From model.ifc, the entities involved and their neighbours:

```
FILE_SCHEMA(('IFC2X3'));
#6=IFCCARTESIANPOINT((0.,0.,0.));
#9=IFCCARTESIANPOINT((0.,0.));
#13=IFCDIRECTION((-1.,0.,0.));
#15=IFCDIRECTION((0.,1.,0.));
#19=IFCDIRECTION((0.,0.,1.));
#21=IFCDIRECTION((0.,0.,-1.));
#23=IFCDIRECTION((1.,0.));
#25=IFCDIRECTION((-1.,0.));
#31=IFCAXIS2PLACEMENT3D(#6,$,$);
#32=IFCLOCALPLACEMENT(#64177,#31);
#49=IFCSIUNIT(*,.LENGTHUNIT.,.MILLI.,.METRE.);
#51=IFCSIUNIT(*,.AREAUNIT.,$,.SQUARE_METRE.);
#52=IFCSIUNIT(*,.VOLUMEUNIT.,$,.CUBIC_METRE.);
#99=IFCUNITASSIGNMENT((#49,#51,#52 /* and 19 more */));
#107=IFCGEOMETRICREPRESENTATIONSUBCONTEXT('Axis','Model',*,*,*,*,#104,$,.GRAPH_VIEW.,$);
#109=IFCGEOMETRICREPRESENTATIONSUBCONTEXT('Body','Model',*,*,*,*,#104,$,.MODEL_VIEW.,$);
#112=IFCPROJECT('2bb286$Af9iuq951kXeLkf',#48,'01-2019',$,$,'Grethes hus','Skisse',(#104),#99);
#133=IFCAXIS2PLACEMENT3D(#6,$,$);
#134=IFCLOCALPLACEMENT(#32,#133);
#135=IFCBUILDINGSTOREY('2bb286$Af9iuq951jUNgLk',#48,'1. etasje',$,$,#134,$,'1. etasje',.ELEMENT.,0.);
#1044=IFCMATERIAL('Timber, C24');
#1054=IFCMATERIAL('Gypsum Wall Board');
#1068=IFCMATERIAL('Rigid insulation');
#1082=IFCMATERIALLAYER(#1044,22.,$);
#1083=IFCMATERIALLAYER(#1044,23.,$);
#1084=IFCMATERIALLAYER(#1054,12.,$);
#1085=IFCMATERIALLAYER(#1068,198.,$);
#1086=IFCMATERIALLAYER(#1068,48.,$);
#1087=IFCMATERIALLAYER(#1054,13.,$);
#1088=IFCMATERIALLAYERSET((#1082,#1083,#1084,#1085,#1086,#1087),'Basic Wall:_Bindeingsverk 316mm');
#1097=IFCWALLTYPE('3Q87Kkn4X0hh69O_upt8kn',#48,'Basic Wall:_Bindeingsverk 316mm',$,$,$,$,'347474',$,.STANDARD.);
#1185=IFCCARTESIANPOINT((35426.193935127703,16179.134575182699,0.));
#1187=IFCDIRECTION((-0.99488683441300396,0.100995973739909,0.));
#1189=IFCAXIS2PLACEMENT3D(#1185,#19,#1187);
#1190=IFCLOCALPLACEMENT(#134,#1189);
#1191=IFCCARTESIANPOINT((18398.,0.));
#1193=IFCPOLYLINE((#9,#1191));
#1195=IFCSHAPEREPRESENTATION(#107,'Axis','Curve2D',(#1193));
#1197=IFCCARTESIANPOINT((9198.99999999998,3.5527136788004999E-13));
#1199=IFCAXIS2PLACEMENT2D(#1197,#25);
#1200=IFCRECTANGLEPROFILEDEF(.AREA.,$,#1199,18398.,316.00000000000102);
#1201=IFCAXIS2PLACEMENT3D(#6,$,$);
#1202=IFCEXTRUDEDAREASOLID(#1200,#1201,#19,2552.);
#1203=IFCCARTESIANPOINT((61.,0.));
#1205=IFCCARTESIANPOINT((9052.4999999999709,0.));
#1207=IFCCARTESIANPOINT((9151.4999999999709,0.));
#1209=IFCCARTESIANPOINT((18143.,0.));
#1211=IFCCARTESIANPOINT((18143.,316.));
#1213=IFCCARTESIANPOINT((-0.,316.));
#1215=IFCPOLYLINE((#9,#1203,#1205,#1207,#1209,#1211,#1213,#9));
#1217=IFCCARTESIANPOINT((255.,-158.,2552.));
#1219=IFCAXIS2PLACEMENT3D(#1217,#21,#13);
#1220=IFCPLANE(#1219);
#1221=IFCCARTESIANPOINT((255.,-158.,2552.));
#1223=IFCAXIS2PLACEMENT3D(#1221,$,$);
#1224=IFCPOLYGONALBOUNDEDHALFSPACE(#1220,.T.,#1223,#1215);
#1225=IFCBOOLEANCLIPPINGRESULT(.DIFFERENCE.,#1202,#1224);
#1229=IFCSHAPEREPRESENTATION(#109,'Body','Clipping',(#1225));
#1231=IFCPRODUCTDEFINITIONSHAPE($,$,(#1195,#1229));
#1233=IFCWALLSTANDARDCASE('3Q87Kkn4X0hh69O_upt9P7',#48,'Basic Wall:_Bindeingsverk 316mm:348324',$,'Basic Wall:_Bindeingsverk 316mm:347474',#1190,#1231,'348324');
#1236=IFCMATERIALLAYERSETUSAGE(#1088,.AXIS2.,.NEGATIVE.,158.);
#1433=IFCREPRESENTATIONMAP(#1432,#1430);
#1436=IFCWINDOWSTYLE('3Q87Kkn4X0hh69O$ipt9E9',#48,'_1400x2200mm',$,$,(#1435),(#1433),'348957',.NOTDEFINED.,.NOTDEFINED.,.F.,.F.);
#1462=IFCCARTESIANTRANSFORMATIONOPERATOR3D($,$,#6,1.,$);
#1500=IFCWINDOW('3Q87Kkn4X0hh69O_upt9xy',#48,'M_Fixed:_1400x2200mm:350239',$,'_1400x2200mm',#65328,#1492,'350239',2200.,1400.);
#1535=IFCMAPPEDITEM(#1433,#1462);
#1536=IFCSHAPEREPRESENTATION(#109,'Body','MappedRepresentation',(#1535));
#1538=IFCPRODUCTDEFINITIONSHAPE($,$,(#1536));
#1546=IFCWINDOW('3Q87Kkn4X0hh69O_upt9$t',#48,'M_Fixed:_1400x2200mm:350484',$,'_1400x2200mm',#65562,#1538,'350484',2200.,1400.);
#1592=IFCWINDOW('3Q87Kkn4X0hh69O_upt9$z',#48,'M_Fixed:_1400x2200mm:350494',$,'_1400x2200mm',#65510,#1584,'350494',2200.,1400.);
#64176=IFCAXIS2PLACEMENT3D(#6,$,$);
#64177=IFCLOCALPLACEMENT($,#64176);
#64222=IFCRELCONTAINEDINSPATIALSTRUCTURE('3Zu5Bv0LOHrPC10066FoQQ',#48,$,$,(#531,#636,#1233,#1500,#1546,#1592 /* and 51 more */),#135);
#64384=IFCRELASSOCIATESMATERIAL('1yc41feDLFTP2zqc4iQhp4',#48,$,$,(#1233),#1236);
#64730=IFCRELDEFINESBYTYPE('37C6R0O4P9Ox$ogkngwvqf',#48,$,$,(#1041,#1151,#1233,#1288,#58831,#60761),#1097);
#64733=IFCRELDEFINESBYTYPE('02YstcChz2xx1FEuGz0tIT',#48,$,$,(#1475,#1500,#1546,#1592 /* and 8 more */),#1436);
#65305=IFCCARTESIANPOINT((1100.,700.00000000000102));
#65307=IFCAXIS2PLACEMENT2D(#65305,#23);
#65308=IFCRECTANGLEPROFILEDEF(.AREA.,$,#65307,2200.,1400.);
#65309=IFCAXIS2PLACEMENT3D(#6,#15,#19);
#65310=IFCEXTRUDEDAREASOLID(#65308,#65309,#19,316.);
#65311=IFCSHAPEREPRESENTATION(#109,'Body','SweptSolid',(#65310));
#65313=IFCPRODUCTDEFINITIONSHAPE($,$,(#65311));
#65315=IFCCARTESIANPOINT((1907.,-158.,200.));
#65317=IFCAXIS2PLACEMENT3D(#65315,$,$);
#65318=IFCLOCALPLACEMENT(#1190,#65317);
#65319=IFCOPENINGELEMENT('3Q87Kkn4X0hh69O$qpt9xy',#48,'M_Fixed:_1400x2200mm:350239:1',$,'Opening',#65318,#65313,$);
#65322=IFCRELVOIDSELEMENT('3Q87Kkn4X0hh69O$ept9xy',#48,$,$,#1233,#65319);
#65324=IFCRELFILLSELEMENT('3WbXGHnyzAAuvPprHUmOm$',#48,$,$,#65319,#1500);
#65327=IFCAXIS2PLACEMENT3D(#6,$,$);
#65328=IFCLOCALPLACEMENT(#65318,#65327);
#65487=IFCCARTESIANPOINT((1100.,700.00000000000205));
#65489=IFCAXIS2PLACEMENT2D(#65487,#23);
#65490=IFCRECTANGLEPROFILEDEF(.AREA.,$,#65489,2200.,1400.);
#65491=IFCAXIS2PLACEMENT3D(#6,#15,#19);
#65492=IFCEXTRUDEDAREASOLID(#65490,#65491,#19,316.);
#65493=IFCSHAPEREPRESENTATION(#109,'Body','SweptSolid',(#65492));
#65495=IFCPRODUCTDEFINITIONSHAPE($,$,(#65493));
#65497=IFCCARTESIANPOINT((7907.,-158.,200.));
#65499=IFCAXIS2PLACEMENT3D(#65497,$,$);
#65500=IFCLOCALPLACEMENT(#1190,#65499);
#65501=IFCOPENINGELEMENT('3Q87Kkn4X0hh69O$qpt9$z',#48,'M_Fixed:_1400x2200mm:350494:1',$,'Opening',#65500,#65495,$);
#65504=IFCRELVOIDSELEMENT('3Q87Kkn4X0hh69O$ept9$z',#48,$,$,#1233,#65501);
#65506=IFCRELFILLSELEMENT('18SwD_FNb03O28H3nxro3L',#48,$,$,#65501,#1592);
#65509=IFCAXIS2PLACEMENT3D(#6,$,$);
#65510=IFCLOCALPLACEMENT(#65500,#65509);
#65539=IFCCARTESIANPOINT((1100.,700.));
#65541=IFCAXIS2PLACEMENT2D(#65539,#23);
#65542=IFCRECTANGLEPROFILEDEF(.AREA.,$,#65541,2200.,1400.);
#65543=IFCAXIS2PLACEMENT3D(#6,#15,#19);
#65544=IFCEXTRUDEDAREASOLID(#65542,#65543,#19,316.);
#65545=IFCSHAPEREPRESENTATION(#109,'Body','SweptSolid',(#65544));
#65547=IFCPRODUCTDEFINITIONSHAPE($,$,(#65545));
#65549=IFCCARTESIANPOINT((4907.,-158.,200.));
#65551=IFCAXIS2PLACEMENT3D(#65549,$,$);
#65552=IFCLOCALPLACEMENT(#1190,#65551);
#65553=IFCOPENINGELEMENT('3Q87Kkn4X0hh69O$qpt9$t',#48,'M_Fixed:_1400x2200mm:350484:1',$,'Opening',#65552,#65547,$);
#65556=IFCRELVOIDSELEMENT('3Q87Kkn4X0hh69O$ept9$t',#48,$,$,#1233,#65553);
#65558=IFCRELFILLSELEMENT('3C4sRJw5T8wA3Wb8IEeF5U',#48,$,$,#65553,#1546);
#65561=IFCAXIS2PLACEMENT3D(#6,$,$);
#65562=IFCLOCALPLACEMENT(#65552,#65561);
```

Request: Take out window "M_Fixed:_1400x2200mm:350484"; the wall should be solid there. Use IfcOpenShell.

```python
import ifcopenshell
import ifcopenshell.api.feature
import ifcopenshell.api.root
import ifcopenshell.geom
import ifcopenshell.util.shape

model = ifcopenshell.open("model.ifc")
settings = ifcopenshell.geom.settings()


def volume(element):
    """Net volume in cubic metres, openings subtracted."""
    shape = ifcopenshell.geom.create_shape(settings, element)
    return ifcopenshell.util.shape.get_volume(shape.geometry)


window = model.by_guid("3Q87Kkn4X0hh69O_upt9$t")
opening = window.FillsVoids[0].RelatingOpeningElement
wall = opening.VoidsElements[0].RelatingBuildingElement
before = volume(wall)

ifcopenshell.api.root.remove_product(model, product=window)
ifcopenshell.api.feature.remove_feature(model, feature=opening)

after = volume(wall)

print(f"wall volume {before:.3f} -> {after:.3f} m3")

model.write("model_rev.ifc")
```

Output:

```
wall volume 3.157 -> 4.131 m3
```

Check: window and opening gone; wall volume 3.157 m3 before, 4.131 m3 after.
